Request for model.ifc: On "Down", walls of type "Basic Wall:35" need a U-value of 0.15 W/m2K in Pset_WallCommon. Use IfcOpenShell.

First a look at what the model holds.

```python
import ifcopenshell
import ifcopenshell.util.element

model = ifcopenshell.open("model.ifc")
print(model.schema)
storey = next(s for s in model.by_type("IfcBuildingStorey") if s.Name == "Down")
walls = [e for e in ifcopenshell.util.element.get_decomposition(storey) if e.is_a("IfcWall")]
seen = {}
for e in walls:
    element_type = ifcopenshell.util.element.get_type(e)
    key = (element_type.Name if element_type != e and element_type else None, ifcopenshell.util.element.get_pset(e, "Pset_WallCommon", "ThermalTransmittance"))
    seen[key] = seen.get(key, 0) + 1
for (name, value), count in sorted(seen.items(), key=str):
    print(count, "x", name, "|", value)
```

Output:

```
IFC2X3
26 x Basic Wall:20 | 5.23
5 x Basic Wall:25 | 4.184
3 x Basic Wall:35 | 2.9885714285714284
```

```python
import ifcopenshell
import ifcopenshell.api.pset
import ifcopenshell.util.element

model = ifcopenshell.open("model.ifc")

storey = next(s for s in model.by_type("IfcBuildingStorey") if s.Name == "Down")
walls = [e for e in ifcopenshell.util.element.get_decomposition(storey) if e.is_a("IfcWall")]

count = 0
for e in walls:
    element_type = ifcopenshell.util.element.get_type(e)
    if element_type in (None, e) or element_type.Name != "Basic Wall:35":
        continue
    # add_pset returns the element's existing set when there is one.
    pset = ifcopenshell.api.pset.add_pset(model, product=e, name="Pset_WallCommon")
    ifcopenshell.api.pset.edit_pset(model, pset=pset, properties={"ThermalTransmittance": 0.15})
    count += 1

print(count, "walls updated")

model.write("model_edited.ifc")
```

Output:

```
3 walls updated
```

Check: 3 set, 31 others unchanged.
